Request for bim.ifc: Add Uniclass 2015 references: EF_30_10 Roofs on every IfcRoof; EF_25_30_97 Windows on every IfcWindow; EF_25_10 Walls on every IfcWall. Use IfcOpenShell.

First a look at what the model holds.

```python
import ifcopenshell

model = ifcopenshell.open("bim.ifc")
print(model.schema)
print("classifications:", [c.Name for c in model.by_type("IfcClassification")])
for ifc_class in ("IfcDoor", "IfcRoof", "IfcStair", "IfcWall", "IfcWindow"):
    print(ifc_class, len(model.by_type(ifc_class)))
```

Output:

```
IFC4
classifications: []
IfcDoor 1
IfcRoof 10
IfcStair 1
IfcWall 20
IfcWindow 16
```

```python
import ifcopenshell
import ifcopenshell.api.classification

model = ifcopenshell.open("bim.ifc")

system = ifcopenshell.api.classification.add_classification(model, classification="Uniclass 2015")

codes = {
    "IfcRoof": ("EF_30_10", "Roofs"),
    "IfcWindow": ("EF_25_30_97", "Windows"),
    "IfcWall": ("EF_25_10", "Walls"),
}
for ifc_class, (code, name) in codes.items():
    products = model.by_type(ifc_class)
    ifcopenshell.api.classification.add_reference(
        model, products=products, classification=system, identification=code, name=name
    )
    print(code, len(products))

model.write("bim_edited.ifc")
```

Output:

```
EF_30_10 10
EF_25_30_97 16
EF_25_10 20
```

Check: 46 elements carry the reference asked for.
